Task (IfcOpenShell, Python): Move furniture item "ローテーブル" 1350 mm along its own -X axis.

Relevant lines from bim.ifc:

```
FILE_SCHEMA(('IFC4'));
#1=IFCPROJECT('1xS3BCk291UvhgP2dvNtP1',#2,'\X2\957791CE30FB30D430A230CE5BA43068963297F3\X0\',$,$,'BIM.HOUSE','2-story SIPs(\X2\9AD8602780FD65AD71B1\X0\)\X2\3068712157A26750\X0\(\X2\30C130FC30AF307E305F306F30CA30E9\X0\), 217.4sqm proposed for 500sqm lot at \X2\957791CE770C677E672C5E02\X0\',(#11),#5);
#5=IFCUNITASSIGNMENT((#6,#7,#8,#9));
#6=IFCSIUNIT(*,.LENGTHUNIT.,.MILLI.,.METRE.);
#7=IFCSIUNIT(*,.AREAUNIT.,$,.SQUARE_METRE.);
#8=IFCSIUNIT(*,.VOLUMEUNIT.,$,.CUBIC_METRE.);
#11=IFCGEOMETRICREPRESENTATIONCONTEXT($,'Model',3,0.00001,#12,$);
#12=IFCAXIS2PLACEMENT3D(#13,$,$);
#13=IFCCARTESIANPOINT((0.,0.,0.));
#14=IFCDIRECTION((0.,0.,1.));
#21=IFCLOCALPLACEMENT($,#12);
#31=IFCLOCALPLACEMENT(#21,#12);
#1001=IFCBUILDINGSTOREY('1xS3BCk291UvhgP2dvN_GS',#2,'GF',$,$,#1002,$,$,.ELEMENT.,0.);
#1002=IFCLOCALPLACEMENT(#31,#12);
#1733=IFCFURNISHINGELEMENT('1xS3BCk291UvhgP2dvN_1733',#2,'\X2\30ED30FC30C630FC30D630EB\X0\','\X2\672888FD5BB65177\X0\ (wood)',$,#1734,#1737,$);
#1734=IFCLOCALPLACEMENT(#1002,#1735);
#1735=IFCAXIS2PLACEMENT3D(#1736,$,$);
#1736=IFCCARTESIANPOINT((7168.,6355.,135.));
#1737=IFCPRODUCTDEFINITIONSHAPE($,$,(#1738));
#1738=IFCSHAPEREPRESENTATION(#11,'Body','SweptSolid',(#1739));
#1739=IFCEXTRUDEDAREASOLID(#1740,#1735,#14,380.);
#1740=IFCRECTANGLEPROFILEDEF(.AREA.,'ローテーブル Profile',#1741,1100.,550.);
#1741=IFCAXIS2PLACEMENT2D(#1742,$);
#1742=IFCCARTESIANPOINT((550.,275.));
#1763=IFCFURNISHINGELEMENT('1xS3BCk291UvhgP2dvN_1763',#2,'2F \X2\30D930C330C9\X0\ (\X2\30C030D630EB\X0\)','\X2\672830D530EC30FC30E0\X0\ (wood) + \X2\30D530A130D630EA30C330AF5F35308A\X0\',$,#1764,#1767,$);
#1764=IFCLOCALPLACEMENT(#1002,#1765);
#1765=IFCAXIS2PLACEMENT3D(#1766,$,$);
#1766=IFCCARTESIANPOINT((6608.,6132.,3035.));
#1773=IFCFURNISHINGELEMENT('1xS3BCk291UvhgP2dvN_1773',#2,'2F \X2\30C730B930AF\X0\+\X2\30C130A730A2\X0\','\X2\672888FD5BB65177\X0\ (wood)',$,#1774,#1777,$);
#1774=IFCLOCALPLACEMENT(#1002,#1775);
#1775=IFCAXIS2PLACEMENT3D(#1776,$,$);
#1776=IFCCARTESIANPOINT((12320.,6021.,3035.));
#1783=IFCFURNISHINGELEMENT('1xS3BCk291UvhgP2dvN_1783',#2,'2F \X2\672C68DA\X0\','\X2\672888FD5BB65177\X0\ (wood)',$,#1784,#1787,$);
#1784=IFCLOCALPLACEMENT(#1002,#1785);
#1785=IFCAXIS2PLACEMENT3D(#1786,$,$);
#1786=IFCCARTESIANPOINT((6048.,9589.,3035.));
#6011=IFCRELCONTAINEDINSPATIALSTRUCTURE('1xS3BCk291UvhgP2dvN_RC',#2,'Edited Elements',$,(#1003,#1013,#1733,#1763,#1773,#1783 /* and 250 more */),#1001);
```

```python
import ifcopenshell
import ifcopenshell.api.geometry
import ifcopenshell.util.placement
import ifcopenshell.util.unit

model = ifcopenshell.open("bim.ifc")
unit_scale = ifcopenshell.util.unit.calculate_unit_scale(model)

item = model.by_id(1733)
matrix = ifcopenshell.util.placement.get_local_placement(item.ObjectPlacement)
matrix[:3, 3] -= matrix[:3, 0] * 1.35 / unit_scale
ifcopenshell.api.geometry.edit_object_placement(model, product=item, matrix=matrix, is_si=False)

print(ifcopenshell.util.placement.get_local_placement(item.ObjectPlacement).round(3) + 0.0)

model.write("bim_updated.ifc")
```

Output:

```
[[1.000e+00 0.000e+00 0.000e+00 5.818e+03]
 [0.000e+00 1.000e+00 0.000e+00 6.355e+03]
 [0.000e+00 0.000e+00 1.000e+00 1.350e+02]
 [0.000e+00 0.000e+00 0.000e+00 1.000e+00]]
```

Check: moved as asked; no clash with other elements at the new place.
